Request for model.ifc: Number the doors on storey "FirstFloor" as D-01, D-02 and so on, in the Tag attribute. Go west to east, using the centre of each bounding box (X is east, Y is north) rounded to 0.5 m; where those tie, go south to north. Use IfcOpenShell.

First a look at what the model holds.

```python
import ifcopenshell
import ifcopenshell.util.element
import ifcopenshell.util.placement

model = ifcopenshell.open("model.ifc")
print(model.schema)
storey = next(s for s in model.by_type("IfcBuildingStorey") if s.Name == "FirstFloor")
doors = [e for e in ifcopenshell.util.element.get_decomposition(storey) if e.is_a("IfcDoor")]
for e in sorted(doors, key=lambda e: e.id()):
    origin = ifcopenshell.util.placement.get_local_placement(e.ObjectPlacement)[:3, 3]
    print(e.id(), e.Tag, e.Name, origin.round(2) + 0.0, sep=" | ")
```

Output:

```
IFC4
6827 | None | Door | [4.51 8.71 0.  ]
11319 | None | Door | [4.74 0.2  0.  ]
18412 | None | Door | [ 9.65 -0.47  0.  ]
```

```python
import ifcopenshell
import ifcopenshell.geom
import ifcopenshell.util.element
import ifcopenshell.util.shape

model = ifcopenshell.open("model.ifc")
settings = ifcopenshell.geom.settings()
settings.set("use-world-coords", True)


def centre(element):
    shape = ifcopenshell.geom.create_shape(settings, element)
    return ifcopenshell.util.shape.get_bbox_centroid(shape.geometry)


storey = next(s for s in model.by_type("IfcBuildingStorey") if s.Name == "FirstFloor")
doors = [e for e in ifcopenshell.util.element.get_decomposition(storey) if e.is_a("IfcDoor")]

# Insertion points can sit at a corner or the storey origin, so sort by the geometry (in metres).
centres = {e: centre(e) for e in doors}
doors.sort(key=lambda e: (round(centres[e][0] / 0.5), centres[e][1]))

for i, e in enumerate(doors, start=1):
    number = f"D-{i:02d}"
    e.Tag = number
    print(e.id(), number)

model.write("model_rev.ifc")
```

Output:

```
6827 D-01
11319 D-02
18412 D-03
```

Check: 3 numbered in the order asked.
